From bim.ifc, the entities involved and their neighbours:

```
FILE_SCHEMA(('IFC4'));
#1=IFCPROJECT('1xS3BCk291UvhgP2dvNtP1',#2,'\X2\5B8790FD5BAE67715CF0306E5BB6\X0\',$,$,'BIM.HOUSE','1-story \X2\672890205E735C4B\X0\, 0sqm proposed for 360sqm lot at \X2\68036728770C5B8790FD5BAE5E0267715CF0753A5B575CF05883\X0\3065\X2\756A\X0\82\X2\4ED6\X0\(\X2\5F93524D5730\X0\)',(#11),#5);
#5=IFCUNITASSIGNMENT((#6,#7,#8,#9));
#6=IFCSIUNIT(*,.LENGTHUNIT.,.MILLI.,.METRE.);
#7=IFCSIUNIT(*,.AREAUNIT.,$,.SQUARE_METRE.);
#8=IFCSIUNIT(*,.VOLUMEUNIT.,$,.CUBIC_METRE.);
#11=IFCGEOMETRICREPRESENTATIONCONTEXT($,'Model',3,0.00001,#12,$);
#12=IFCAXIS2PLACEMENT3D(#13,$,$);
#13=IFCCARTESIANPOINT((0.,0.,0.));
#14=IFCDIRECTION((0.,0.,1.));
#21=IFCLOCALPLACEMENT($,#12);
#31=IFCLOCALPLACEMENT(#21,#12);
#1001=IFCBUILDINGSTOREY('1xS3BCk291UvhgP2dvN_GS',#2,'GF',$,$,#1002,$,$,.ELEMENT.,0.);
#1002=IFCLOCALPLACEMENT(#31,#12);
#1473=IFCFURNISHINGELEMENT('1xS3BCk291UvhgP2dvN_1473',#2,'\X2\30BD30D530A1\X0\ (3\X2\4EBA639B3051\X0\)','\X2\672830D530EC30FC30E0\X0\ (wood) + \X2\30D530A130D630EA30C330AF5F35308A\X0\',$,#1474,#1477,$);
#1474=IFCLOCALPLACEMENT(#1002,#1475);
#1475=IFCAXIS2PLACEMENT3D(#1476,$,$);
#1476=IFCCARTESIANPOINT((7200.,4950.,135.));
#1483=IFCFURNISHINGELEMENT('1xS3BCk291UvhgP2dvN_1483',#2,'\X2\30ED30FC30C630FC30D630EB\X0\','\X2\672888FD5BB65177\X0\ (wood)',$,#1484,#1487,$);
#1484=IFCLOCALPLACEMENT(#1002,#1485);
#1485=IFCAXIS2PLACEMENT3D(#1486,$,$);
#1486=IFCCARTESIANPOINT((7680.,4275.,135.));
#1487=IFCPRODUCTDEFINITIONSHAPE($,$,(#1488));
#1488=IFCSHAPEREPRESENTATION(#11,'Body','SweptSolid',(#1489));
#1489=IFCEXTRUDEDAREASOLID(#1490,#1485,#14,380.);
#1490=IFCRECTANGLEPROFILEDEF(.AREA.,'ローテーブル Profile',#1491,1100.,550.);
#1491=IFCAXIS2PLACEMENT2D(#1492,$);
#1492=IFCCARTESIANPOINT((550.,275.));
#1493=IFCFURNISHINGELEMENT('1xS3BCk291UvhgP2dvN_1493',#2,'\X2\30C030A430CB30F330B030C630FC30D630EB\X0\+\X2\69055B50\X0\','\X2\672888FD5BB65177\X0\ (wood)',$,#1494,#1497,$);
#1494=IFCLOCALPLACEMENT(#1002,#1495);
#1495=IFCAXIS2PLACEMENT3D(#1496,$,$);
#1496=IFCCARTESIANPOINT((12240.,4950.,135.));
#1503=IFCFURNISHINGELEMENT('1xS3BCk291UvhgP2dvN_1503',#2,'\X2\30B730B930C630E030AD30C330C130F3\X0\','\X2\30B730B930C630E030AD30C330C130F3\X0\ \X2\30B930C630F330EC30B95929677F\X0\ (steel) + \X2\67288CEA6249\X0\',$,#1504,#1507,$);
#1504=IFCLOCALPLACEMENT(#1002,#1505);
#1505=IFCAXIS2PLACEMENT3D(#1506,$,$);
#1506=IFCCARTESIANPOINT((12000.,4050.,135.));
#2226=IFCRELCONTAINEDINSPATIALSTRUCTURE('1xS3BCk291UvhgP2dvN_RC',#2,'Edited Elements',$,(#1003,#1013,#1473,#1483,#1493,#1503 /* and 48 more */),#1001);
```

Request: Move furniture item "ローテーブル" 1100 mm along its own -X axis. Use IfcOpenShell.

```python
import ifcopenshell
import ifcopenshell.api.geometry
import ifcopenshell.util.placement

model = ifcopenshell.open("bim.ifc")

item = model.by_guid("1xS3BCk291UvhgP2dvN_1483")
matrix = ifcopenshell.util.placement.get_local_placement(item.ObjectPlacement)
matrix[:3, 3] -= matrix[:3, 0] * 1100.0
ifcopenshell.api.geometry.edit_object_placement(model, product=item, matrix=matrix, is_si=False)

print(ifcopenshell.util.placement.get_local_placement(item.ObjectPlacement).round(3) + 0.0)

model.write("bim_v2.ifc")
```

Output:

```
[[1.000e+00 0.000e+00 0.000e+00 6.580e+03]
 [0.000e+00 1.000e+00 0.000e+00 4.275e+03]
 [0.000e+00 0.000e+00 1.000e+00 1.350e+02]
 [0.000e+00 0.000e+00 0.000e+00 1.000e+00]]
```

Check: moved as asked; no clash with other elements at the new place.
